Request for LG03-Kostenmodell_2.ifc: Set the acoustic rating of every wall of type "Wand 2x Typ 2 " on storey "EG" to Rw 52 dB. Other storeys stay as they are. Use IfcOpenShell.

First a look at what the model holds.

```python
import ifcopenshell
import ifcopenshell.util.element

model = ifcopenshell.open("LG03-Kostenmodell_2.ifc")
print(model.schema)
storey = next(s for s in model.by_type("IfcBuildingStorey") if s.Name == "EG")
walls = [e for e in ifcopenshell.util.element.get_decomposition(storey) if e.is_a("IfcWall")]
seen = {}
for e in walls:
    element_type = ifcopenshell.util.element.get_type(e)
    key = (element_type.Name if element_type != e and element_type else None, ifcopenshell.util.element.get_pset(e, "Pset_WallCommon", "AcousticRating"))
    seen[key] = seen.get(key, 0) + 1
for (name, value), count in sorted(seen.items(), key=str):
    print(count, "x", name, "|", value)
```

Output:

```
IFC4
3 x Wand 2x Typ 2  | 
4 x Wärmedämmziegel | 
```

```python
import ifcopenshell
import ifcopenshell.api.pset
import ifcopenshell.util.element

model = ifcopenshell.open("LG03-Kostenmodell_2.ifc")

storey = next(s for s in model.by_type("IfcBuildingStorey") if s.Name == "EG")
walls = [e for e in ifcopenshell.util.element.get_decomposition(storey) if e.is_a("IfcWall")]

count = 0
for e in walls:
    element_type = ifcopenshell.util.element.get_type(e)
    if element_type in (None, e) or element_type.Name != "Wand 2x Typ 2 ":
        continue
    # add_pset returns the element's existing set when there is one.
    pset = ifcopenshell.api.pset.add_pset(model, product=e, name="Pset_WallCommon")
    ifcopenshell.api.pset.edit_pset(model, pset=pset, properties={"AcousticRating": "Rw 52 dB"})
    count += 1

print(count, "walls updated")

model.write("LG03-Kostenmodell_2_edited.ifc")
```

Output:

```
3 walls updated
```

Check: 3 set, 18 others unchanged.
